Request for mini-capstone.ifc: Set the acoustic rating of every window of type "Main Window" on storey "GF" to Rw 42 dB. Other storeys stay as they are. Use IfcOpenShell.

First a look at what the model holds.

```python
import ifcopenshell
import ifcopenshell.util.element

model = ifcopenshell.open("mini-capstone.ifc")
print(model.schema)
storey = next(s for s in model.by_type("IfcBuildingStorey") if s.Name == "GF")
windows = [e for e in ifcopenshell.util.element.get_decomposition(storey) if e.is_a("IfcWindow")]
seen = {}
for e in windows:
    element_type = ifcopenshell.util.element.get_type(e)
    key = (element_type.Name if element_type != e and element_type else None, ifcopenshell.util.element.get_pset(e, "Pset_WindowCommon", "AcousticRating"))
    seen[key] = seen.get(key, 0) + 1
for (name, value), count in sorted(seen.items(), key=str):
    print(count, "x", name, "|", value)
```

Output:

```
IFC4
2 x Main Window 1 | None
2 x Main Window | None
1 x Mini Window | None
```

```python
import ifcopenshell
import ifcopenshell.api.pset
import ifcopenshell.util.element

model = ifcopenshell.open("mini-capstone.ifc")

storey = next(s for s in model.by_type("IfcBuildingStorey") if s.Name == "GF")
windows = [e for e in ifcopenshell.util.element.get_decomposition(storey) if e.is_a("IfcWindow")]

count = 0
for e in windows:
    element_type = ifcopenshell.util.element.get_type(e)
    if element_type in (None, e) or element_type.Name != "Main Window":
        continue
    # add_pset returns the element's existing set when there is one.
    pset = ifcopenshell.api.pset.add_pset(model, product=e, name="Pset_WindowCommon")
    ifcopenshell.api.pset.edit_pset(model, pset=pset, properties={"AcousticRating": "Rw 42 dB"})
    count += 1

print(count, "windows updated")

model.write("mini-capstone_v2.ifc")
```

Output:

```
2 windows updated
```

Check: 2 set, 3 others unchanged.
